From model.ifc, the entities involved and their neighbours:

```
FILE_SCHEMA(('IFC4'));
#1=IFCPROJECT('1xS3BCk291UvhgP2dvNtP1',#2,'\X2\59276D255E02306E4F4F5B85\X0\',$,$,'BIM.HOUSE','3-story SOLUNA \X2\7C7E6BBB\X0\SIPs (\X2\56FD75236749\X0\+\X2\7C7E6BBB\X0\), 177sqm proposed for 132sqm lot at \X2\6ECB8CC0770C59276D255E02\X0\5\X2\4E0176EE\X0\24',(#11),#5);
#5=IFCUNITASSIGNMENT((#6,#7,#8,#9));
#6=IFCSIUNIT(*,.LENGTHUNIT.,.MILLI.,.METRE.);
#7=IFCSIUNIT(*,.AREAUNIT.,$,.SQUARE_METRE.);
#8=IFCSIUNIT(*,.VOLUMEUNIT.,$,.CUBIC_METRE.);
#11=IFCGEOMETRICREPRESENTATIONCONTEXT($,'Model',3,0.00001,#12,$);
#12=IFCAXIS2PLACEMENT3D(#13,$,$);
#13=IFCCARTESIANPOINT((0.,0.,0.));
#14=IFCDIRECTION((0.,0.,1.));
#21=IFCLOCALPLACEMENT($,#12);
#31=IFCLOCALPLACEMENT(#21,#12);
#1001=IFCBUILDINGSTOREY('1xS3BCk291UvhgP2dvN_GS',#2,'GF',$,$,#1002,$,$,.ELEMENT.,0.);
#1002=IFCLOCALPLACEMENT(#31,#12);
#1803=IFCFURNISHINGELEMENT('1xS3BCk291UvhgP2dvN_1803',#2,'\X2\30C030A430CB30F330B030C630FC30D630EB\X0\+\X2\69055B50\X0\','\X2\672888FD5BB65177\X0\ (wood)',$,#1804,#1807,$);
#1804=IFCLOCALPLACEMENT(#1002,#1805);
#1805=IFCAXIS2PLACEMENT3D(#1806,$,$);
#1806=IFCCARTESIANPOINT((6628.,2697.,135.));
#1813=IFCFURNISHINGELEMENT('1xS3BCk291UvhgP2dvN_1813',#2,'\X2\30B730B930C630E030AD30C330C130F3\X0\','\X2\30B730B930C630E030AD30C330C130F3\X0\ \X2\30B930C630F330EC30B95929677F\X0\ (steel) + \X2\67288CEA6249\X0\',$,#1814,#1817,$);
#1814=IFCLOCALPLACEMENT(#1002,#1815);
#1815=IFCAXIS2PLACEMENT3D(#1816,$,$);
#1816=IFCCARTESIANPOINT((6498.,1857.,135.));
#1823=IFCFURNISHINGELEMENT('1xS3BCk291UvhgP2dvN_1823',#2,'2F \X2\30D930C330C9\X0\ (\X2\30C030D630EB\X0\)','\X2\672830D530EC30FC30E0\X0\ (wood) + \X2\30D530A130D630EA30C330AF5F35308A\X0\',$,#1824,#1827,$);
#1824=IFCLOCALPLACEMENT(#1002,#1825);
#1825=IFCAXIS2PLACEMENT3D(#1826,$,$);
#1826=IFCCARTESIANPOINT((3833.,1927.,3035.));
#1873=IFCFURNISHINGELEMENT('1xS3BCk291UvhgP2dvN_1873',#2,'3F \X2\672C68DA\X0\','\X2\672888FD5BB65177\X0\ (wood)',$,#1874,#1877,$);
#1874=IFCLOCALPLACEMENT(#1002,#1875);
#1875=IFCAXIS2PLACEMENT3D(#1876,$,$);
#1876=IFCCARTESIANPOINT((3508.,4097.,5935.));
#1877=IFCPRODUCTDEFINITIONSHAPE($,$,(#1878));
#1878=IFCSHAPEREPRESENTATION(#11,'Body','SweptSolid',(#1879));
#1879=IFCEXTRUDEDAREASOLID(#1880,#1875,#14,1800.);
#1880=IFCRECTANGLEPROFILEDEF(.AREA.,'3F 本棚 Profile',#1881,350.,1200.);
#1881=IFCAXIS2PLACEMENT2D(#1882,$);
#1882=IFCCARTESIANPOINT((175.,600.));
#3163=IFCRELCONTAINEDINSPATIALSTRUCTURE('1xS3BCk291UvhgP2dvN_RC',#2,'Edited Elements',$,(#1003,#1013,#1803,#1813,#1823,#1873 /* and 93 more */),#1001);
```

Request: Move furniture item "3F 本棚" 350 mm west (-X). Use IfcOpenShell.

```python
import ifcopenshell
import ifcopenshell.api.geometry
import ifcopenshell.util.placement

model = ifcopenshell.open("model.ifc")

item = model.by_guid("1xS3BCk291UvhgP2dvN_1873")
matrix = ifcopenshell.util.placement.get_local_placement(item.ObjectPlacement)
matrix[0, 3] -= 350.0
ifcopenshell.api.geometry.edit_object_placement(model, product=item, matrix=matrix, is_si=False)

print(ifcopenshell.util.placement.get_local_placement(item.ObjectPlacement).round(3) + 0.0)

model.write("model-out.ifc")
```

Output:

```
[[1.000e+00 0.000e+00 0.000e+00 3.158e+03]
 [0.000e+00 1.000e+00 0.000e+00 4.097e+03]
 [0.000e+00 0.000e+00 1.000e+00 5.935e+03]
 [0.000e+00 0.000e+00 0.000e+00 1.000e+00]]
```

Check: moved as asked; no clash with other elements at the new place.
